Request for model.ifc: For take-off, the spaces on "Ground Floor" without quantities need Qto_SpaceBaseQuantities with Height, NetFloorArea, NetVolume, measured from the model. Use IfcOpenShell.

First a look at what the model holds.

```python
import ifcopenshell
import ifcopenshell.util.element
import ifcopenshell.util.unit

model = ifcopenshell.open("model.ifc")
print(model.schema)
for unit_type in ("LENGTHUNIT", "AREAUNIT", "VOLUMEUNIT"):
    print(unit_type, ifcopenshell.util.unit.calculate_unit_scale(model, unit_type))
storey = next(s for s in model.by_type("IfcBuildingStorey") if s.Name == "Ground Floor")
spaces = [e for e in ifcopenshell.util.element.get_decomposition(storey) if e.is_a("IfcSpace")]
for e in sorted(spaces, key=lambda e: e.id()):
    print(e.id(), e.is_a(), e.Name, list(ifcopenshell.util.element.get_psets(e, qtos_only=True)), sep=" | ")
```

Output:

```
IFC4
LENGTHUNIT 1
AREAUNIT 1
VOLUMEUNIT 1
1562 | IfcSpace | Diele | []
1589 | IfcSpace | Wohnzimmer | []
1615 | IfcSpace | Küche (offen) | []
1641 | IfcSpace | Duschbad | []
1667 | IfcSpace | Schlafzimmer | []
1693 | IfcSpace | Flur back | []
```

```python
import ifcopenshell
import ifcopenshell.api.pset
import ifcopenshell.geom
import ifcopenshell.util.element
import ifcopenshell.util.shape
import ifcopenshell.util.unit

model = ifcopenshell.open("model.ifc")
unit_scale = ifcopenshell.util.unit.calculate_unit_scale(model)
area_scale = ifcopenshell.util.unit.calculate_unit_scale(model, "AREAUNIT")
volume_scale = ifcopenshell.util.unit.calculate_unit_scale(model, "VOLUMEUNIT")
settings = ifcopenshell.geom.settings()

storey = next(s for s in model.by_type("IfcBuildingStorey") if s.Name == "Ground Floor")
spaces = [e for e in ifcopenshell.util.element.get_decomposition(storey) if e.is_a("IfcSpace")]

for e in sorted(spaces, key=lambda e: e.id()):
    if ifcopenshell.util.element.get_psets(e, qtos_only=True, should_inherit=False):
        continue
    # Geometry comes back in metres, in the element's own axes.
    shape = ifcopenshell.geom.create_shape(settings, e)
    values = {
        "Height": ifcopenshell.util.shape.get_z(shape.geometry) / unit_scale,
        "NetFloorArea": ifcopenshell.util.shape.get_footprint_area(shape.geometry) / area_scale,
        "NetVolume": ifcopenshell.util.shape.get_volume(shape.geometry) / volume_scale,
    }
    qto = ifcopenshell.api.pset.add_qto(model, product=e, name="Qto_SpaceBaseQuantities")
    ifcopenshell.api.pset.edit_qto(model, qto=qto, properties=values)
    print(e.id(), {k: round(v, 3) for k, v in values.items()})

model.write("model_v2.ifc")
```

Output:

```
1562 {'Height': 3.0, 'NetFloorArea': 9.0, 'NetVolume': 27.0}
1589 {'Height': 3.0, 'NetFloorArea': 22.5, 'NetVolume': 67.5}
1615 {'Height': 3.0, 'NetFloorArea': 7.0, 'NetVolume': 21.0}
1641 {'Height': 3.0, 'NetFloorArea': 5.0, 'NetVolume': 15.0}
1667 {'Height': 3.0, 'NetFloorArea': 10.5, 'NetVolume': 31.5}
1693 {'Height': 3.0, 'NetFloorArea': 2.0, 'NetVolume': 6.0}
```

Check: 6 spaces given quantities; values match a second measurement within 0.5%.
